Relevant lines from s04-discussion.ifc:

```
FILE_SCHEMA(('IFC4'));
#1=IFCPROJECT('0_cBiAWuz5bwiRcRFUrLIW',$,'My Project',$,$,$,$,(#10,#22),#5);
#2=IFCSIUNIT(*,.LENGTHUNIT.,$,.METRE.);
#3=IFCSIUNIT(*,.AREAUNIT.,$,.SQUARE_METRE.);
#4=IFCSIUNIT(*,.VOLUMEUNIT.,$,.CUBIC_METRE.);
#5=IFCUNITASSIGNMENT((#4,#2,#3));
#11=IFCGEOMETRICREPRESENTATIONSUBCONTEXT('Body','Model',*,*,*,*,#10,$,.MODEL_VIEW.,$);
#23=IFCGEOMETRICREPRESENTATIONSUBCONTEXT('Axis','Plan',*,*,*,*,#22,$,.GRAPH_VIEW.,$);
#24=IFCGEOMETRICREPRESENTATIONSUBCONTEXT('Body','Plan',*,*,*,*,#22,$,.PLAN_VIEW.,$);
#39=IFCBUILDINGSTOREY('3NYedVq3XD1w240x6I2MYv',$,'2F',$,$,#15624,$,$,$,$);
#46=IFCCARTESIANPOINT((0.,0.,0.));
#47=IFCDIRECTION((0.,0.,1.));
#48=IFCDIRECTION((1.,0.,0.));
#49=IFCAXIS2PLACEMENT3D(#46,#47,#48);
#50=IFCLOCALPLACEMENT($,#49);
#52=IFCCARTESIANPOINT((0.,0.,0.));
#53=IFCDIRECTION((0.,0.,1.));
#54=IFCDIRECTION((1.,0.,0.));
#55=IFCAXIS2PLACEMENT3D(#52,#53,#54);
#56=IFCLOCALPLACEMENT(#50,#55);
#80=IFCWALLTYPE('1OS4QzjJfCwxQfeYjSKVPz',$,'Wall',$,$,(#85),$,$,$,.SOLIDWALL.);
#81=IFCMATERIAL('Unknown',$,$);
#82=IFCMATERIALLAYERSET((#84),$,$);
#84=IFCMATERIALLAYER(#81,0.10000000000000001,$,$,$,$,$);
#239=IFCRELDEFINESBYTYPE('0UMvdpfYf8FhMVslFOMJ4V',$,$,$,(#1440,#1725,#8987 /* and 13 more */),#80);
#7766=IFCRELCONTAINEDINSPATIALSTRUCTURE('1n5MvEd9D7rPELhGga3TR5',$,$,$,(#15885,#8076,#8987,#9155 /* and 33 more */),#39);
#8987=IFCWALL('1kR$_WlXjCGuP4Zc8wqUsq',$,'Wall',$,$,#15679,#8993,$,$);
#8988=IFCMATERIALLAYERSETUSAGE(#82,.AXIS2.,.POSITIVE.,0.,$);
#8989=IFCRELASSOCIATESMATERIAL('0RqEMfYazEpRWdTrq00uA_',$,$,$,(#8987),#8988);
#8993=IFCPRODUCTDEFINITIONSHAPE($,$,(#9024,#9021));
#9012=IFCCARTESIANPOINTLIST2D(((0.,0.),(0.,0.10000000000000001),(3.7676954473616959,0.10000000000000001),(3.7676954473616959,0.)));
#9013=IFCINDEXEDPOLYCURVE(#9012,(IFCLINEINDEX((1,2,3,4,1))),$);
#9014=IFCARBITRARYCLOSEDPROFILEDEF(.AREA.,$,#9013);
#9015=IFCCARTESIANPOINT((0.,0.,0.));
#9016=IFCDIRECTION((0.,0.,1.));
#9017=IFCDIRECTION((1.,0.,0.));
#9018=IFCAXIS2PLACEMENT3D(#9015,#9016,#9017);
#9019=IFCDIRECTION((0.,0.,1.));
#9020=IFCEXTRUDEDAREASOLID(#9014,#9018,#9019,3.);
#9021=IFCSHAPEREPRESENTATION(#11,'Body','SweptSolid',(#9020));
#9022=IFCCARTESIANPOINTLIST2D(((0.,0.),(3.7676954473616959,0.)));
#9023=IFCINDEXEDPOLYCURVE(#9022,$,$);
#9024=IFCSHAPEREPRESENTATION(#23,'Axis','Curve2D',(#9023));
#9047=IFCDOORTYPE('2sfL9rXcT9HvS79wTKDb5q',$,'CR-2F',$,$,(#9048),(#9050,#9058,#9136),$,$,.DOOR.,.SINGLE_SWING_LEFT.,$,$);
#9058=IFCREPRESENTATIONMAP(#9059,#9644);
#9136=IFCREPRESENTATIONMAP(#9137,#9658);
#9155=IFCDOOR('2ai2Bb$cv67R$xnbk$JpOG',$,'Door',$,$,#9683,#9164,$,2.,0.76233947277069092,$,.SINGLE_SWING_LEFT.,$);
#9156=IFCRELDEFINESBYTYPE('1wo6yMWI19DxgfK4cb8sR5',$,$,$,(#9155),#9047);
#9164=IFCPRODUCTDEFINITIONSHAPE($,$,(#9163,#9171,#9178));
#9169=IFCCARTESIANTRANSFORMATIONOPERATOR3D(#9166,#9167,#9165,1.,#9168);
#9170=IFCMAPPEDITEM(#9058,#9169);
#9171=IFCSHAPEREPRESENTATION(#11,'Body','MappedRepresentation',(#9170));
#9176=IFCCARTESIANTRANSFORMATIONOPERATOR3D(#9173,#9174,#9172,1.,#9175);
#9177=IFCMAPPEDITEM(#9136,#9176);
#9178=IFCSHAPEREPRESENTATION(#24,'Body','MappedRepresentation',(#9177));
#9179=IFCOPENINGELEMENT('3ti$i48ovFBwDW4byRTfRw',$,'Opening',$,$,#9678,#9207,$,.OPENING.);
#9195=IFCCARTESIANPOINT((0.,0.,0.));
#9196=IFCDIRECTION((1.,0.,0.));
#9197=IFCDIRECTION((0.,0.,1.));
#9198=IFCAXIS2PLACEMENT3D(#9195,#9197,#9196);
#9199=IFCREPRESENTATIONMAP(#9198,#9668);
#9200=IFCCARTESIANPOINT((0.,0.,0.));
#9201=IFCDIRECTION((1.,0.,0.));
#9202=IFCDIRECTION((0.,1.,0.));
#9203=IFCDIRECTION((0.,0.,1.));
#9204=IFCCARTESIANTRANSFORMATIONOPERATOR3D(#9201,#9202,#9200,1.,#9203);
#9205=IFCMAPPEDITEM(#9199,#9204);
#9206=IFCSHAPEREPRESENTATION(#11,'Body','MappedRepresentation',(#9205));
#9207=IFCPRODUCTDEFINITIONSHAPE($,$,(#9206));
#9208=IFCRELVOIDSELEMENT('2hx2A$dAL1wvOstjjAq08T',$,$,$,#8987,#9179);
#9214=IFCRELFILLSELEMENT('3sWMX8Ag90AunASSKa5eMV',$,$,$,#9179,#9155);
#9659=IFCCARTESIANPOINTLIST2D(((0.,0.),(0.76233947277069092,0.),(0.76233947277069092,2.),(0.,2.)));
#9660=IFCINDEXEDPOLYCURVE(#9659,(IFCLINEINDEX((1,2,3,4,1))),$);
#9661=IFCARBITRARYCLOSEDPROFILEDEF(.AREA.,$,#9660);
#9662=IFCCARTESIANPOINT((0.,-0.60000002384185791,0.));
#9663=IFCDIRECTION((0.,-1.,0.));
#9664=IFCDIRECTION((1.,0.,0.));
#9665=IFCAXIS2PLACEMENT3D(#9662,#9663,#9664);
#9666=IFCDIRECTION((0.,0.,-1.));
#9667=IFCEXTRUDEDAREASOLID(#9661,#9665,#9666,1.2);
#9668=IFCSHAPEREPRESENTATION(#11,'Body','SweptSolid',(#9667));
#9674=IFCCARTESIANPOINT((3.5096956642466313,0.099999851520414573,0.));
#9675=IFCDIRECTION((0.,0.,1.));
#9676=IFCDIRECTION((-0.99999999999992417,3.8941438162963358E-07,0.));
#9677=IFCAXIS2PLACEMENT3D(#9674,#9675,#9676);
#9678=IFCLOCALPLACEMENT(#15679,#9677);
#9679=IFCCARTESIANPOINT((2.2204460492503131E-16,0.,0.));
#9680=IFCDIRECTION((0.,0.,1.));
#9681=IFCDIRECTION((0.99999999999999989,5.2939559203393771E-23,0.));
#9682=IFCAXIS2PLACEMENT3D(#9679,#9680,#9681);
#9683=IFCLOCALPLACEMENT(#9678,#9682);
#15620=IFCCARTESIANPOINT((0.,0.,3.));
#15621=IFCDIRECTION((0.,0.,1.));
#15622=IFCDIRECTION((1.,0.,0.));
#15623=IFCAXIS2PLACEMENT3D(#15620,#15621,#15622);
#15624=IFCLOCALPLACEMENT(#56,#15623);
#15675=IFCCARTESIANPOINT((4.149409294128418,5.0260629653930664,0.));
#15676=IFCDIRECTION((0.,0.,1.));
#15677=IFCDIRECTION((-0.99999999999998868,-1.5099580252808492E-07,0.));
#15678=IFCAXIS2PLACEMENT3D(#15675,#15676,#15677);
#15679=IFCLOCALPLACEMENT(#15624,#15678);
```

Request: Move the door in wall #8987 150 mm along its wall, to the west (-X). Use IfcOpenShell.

```python
import ifcopenshell
import ifcopenshell.api.geometry
import ifcopenshell.util.placement

model = ifcopenshell.open("s04-discussion.ifc")

door = model.by_guid("2ai2Bb$cv67R$xnbk$JpOG")
opening = door.FillsVoids[0].RelatingOpeningElement
wall = opening.VoidsElements[0].RelatingBuildingElement

wall_matrix = ifcopenshell.util.placement.get_local_placement(wall.ObjectPlacement)
shift = wall_matrix[:3, 0] * 0.15
before = ifcopenshell.util.placement.get_local_placement(door.ObjectPlacement)[:3, 3].copy()

# The door is placed relative to its opening, so it follows when the opening moves.
matrix = ifcopenshell.util.placement.get_local_placement(opening.ObjectPlacement)
matrix[:3, 3] += shift
ifcopenshell.api.geometry.edit_object_placement(
    model, product=opening, matrix=matrix, is_si=False, should_transform_children=True
)

after = ifcopenshell.util.placement.get_local_placement(door.ObjectPlacement)[:3, 3]
print("door moved by", (after - before).round(3) + 0.0)

model.write("s04-discussion_edited.ifc")
```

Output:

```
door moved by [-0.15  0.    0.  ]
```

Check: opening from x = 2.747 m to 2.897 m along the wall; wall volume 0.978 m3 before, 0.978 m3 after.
